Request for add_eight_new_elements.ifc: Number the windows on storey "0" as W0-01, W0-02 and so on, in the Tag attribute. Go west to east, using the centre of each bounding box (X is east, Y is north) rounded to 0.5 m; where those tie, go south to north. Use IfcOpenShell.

First a look at what the model holds.

```python
import ifcopenshell
import ifcopenshell.util.element
import ifcopenshell.util.placement

model = ifcopenshell.open("add_eight_new_elements.ifc")
print(model.schema)
storey = next(s for s in model.by_type("IfcBuildingStorey") if s.Name == "0")
windows = [e for e in ifcopenshell.util.element.get_decomposition(storey) if e.is_a("IfcWindow")]
for e in sorted(windows, key=lambda e: e.id()):
    origin = ifcopenshell.util.placement.get_local_placement(e.ObjectPlacement)[:3, 3]
    print(e.id(), e.Tag, e.Name, origin.round(2) + 0.0, sep=" | ")
```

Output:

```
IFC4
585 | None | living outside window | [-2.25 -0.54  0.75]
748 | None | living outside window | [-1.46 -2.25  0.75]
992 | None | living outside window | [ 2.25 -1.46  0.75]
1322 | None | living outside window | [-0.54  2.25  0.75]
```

```python
import ifcopenshell
import ifcopenshell.geom
import ifcopenshell.util.element
import ifcopenshell.util.shape

model = ifcopenshell.open("add_eight_new_elements.ifc")
settings = ifcopenshell.geom.settings()
settings.set("use-world-coords", True)


def centre(element):
    shape = ifcopenshell.geom.create_shape(settings, element)
    return ifcopenshell.util.shape.get_bbox_centroid(shape.geometry)


storey = next(s for s in model.by_type("IfcBuildingStorey") if s.Name == "0")
windows = [e for e in ifcopenshell.util.element.get_decomposition(storey) if e.is_a("IfcWindow")]

# Insertion points can sit at a corner or the storey origin, so sort by the geometry (in metres).
centres = {e: centre(e) for e in windows}
windows.sort(key=lambda e: (round(centres[e][0] / 0.5), centres[e][1]))

for i, e in enumerate(windows, start=1):
    number = f"W0-{i:02d}"
    e.Tag = number
    print(e.id(), number)

model.write("add_eight_new_elements_rev.ifc")
```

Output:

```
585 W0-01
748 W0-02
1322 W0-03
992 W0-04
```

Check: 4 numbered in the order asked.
